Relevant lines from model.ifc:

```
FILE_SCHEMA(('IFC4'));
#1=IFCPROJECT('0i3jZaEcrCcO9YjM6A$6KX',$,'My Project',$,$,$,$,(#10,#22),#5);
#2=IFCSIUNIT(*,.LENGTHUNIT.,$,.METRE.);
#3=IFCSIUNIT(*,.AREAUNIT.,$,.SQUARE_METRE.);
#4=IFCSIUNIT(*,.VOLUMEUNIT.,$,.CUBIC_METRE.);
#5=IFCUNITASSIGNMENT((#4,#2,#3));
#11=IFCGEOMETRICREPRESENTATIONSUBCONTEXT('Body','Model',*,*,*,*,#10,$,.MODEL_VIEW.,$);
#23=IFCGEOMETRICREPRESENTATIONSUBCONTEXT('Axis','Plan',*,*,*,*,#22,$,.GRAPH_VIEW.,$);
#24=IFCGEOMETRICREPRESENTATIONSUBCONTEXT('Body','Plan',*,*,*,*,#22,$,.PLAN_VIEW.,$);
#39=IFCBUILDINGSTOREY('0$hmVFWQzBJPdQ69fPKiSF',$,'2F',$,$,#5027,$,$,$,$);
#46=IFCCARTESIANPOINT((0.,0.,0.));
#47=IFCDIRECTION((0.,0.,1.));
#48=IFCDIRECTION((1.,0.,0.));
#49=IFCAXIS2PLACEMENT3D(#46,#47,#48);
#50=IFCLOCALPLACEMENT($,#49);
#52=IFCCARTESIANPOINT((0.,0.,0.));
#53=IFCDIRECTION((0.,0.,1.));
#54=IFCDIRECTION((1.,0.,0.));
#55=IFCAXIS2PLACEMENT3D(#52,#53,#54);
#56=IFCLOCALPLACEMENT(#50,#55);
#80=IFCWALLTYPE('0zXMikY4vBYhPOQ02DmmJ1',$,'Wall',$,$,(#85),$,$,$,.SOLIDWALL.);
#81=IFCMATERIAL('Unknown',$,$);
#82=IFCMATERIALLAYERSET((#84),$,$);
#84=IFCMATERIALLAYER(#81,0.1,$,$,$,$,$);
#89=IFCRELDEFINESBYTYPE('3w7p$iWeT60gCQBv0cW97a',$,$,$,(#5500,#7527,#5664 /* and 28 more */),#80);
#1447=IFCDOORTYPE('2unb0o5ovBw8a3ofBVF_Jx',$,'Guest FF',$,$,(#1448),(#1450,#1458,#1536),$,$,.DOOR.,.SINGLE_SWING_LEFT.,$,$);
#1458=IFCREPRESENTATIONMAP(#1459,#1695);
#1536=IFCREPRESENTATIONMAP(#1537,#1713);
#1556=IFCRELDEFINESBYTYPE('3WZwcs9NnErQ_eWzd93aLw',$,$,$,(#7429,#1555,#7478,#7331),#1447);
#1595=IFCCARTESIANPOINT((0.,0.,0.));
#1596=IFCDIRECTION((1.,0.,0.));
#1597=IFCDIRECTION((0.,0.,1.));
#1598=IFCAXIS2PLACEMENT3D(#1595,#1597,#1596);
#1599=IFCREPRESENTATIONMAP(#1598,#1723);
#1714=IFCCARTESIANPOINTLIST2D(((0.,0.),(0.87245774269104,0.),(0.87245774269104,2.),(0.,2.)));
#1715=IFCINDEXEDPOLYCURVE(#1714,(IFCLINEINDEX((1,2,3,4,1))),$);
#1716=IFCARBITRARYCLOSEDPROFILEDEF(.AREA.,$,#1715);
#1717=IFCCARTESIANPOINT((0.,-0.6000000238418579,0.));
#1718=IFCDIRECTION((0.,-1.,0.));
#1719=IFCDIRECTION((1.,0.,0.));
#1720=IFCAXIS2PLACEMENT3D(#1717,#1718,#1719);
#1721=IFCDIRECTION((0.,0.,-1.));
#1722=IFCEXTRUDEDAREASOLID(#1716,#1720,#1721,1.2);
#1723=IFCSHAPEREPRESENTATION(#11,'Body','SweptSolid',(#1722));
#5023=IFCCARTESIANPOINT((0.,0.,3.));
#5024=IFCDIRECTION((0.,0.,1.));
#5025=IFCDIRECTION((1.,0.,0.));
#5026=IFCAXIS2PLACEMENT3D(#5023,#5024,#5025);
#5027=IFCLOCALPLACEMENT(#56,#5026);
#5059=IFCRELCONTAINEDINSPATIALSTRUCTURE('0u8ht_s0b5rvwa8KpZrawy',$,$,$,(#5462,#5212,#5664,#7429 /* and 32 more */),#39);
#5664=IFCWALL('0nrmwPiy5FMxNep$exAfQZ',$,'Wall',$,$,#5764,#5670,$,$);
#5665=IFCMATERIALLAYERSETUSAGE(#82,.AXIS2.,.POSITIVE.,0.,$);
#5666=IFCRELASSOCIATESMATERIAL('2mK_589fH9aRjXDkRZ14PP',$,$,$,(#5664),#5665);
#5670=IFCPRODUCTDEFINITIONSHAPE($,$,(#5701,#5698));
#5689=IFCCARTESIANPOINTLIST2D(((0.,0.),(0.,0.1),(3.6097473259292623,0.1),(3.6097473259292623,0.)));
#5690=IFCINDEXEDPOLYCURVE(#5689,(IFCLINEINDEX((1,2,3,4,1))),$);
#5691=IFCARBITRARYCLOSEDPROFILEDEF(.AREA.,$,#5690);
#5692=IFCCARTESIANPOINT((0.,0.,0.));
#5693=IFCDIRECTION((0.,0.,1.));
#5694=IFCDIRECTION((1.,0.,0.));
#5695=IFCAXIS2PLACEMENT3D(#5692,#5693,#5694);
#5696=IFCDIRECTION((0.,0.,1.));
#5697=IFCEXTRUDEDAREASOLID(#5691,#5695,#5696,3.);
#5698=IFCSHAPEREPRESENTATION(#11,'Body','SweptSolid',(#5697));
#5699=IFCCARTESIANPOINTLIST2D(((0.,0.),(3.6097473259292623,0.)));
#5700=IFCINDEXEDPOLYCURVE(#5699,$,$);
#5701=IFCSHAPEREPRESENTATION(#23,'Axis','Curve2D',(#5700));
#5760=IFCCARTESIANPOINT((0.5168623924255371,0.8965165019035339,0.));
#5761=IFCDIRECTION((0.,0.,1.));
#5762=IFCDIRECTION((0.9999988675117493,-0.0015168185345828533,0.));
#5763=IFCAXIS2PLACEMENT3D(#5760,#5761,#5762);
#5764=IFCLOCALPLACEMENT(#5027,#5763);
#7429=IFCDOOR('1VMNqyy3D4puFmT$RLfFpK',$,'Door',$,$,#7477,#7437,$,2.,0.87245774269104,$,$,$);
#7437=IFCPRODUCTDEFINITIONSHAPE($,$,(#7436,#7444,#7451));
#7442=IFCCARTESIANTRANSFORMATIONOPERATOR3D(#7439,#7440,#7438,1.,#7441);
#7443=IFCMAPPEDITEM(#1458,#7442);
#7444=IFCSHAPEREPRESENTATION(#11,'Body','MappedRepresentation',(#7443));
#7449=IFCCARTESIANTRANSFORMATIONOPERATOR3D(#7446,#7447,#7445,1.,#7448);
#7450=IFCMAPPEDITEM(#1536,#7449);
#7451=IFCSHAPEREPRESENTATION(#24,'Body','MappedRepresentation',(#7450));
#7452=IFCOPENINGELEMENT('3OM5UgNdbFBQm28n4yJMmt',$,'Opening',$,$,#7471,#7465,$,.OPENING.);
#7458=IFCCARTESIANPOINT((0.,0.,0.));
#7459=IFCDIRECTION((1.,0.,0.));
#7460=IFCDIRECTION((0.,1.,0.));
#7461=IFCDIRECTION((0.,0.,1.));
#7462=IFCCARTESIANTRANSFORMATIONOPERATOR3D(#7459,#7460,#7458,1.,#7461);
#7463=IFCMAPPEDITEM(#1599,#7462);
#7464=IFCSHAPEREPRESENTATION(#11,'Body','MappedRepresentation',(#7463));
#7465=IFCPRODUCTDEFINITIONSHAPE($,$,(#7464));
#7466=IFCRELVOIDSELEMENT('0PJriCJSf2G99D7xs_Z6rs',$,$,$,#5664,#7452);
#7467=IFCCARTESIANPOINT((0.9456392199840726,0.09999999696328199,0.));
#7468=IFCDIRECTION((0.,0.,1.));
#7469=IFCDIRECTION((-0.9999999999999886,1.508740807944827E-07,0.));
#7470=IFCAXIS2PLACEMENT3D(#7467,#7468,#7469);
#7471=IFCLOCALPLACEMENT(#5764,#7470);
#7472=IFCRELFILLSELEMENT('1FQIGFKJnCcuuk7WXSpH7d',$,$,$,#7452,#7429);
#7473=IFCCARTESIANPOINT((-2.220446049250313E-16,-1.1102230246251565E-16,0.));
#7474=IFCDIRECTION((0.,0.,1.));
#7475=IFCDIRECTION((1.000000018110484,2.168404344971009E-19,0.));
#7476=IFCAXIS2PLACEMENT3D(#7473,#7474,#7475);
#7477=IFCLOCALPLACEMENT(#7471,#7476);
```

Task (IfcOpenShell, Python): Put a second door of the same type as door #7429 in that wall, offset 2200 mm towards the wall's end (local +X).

```python
import ifcopenshell
import ifcopenshell.api.feature
import ifcopenshell.api.geometry
import ifcopenshell.api.root
import ifcopenshell.geom
import ifcopenshell.util.element
import ifcopenshell.util.placement
import ifcopenshell.util.shape
import ifcopenshell.util.unit

model = ifcopenshell.open("model.ifc")
unit_scale = ifcopenshell.util.unit.calculate_unit_scale(model)
settings = ifcopenshell.geom.settings()


def volume(element):
    """Net volume in cubic metres, openings subtracted."""
    shape = ifcopenshell.geom.create_shape(settings, element)
    return ifcopenshell.util.shape.get_volume(shape.geometry)


door = model.by_guid("1VMNqyy3D4puFmT$RLfFpK")
opening = door.FillsVoids[0].RelatingOpeningElement
wall = opening.VoidsElements[0].RelatingBuildingElement
before = volume(wall)
shift = ifcopenshell.util.placement.get_local_placement(wall.ObjectPlacement)[:3, 0] * 2.2 / unit_scale

# copy_class copies the void relationship, type, container and properties, but no geometry.
new_opening = ifcopenshell.api.root.copy_class(model, product=opening)
new_opening.Representation = ifcopenshell.util.element.copy_deep(
    model, opening.Representation, exclude=["IfcGeometricRepresentationContext", "IfcRepresentationMap"]
)
new_door = ifcopenshell.api.root.copy_class(model, product=door)
new_door.Representation = ifcopenshell.util.element.copy_deep(
    model, door.Representation, exclude=["IfcGeometricRepresentationContext", "IfcRepresentationMap"]
)
ifcopenshell.api.feature.add_filling(model, opening=new_opening, element=new_door)

for old, new in ((opening, new_opening), (door, new_door)):
    matrix = ifcopenshell.util.placement.get_local_placement(old.ObjectPlacement)
    matrix[:3, 3] += shift
    ifcopenshell.api.geometry.edit_object_placement(model, product=new, matrix=matrix, is_si=False)

after = volume(wall)

print(f"wall volume {before:.3f} -> {after:.3f} m3")

model.write("model_updated.ifc")
```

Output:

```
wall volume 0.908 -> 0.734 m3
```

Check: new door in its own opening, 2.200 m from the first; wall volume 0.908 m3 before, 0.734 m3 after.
